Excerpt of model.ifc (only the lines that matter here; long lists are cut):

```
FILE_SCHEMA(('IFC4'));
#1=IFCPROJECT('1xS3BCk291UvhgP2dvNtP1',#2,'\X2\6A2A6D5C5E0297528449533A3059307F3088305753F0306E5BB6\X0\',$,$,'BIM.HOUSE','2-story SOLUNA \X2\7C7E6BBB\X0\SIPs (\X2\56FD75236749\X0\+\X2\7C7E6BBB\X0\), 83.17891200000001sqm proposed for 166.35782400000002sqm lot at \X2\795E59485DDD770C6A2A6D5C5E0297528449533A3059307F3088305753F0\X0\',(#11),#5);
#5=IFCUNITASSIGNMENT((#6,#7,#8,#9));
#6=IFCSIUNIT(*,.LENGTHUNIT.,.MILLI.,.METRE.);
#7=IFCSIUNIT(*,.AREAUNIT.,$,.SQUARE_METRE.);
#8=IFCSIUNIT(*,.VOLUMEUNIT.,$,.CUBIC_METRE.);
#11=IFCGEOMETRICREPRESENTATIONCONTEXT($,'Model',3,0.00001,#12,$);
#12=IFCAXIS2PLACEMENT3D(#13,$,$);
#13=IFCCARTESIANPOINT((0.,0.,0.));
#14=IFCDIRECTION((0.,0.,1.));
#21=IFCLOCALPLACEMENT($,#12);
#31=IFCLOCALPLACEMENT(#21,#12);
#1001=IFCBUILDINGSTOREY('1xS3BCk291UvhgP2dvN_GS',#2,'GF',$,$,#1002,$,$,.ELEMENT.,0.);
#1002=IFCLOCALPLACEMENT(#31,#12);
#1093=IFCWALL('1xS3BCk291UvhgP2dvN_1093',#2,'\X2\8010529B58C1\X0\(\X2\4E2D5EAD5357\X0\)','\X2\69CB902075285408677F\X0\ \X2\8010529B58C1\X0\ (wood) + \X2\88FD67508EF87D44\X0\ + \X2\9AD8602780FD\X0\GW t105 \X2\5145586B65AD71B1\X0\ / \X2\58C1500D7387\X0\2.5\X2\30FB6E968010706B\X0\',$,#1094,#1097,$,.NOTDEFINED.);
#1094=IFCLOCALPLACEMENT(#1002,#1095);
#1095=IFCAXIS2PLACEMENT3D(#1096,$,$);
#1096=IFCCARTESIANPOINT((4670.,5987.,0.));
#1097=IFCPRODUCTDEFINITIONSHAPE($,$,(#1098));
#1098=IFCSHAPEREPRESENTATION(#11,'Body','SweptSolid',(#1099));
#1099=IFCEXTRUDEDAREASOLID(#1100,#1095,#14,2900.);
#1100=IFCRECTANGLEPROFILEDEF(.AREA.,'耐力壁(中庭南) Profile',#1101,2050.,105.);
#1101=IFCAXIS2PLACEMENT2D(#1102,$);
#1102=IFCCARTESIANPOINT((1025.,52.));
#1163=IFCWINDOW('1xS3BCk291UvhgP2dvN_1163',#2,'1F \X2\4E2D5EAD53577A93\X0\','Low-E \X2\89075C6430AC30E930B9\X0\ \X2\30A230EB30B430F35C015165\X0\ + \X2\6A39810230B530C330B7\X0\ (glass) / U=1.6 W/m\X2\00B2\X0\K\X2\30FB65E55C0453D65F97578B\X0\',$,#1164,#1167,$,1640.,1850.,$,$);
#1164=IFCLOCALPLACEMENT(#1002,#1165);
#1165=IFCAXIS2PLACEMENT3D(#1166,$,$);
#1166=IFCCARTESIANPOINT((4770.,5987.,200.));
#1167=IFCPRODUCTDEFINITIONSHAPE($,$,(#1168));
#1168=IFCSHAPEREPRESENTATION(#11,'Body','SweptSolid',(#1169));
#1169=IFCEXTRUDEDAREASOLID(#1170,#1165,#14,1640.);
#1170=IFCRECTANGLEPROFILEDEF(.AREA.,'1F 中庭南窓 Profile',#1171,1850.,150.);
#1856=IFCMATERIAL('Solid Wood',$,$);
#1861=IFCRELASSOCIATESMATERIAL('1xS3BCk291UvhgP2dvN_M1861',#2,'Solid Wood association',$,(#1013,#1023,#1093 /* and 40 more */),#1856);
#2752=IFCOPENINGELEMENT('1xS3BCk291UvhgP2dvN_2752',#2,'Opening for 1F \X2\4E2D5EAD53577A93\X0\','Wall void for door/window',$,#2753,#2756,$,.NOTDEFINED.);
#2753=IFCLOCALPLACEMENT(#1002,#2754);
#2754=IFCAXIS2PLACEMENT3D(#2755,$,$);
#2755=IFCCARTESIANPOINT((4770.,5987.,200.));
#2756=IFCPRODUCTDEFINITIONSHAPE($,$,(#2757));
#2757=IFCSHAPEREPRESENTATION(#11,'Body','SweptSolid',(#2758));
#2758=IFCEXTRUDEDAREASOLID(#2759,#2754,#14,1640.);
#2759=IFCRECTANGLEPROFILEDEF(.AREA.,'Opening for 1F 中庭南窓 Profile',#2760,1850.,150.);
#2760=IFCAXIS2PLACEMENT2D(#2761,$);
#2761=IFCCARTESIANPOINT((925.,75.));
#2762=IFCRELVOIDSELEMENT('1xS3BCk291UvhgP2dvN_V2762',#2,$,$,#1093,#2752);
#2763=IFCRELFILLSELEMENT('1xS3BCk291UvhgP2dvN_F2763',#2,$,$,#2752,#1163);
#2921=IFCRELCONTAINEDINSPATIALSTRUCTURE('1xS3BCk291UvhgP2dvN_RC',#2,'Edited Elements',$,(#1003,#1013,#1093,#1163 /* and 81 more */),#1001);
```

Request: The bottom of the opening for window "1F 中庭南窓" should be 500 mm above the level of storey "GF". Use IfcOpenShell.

```python
import numpy as np
import ifcopenshell
import ifcopenshell.api.geometry
import ifcopenshell.geom
import ifcopenshell.util.element
import ifcopenshell.util.placement
import ifcopenshell.util.shape
import ifcopenshell.util.unit

model = ifcopenshell.open("model.ifc")
unit_scale = ifcopenshell.util.unit.calculate_unit_scale(model)

window = model.by_guid("1xS3BCk291UvhgP2dvN_1163")
opening = window.FillsVoids[0].RelatingOpeningElement
storey = ifcopenshell.util.element.get_container(window, ifc_class="IfcBuildingStorey")
level = ifcopenshell.util.placement.get_local_placement(storey.ObjectPlacement)[2, 3]

# The opening's origin need not be at the sill, so measure its lowest point.
shape = ifcopenshell.geom.create_shape(ifcopenshell.geom.settings(), opening)
bottom = ifcopenshell.util.shape.get_shape_bottom_elevation(shape, shape.geometry) / unit_scale
dz = level + 500.0 - bottom

shift = np.array([0.0, 0.0, dz])
# The window is not placed relative to its opening, so move both.
for product in (opening, window):
    matrix = ifcopenshell.util.placement.get_local_placement(product.ObjectPlacement)
    matrix[:3, 3] += shift
    ifcopenshell.api.geometry.edit_object_placement(model, product=product, matrix=matrix, is_si=False)

print(f"moved by {dz * unit_scale:+.3f} m")

model.write("model-out.ifc")
```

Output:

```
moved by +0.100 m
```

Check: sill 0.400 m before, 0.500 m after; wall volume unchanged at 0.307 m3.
